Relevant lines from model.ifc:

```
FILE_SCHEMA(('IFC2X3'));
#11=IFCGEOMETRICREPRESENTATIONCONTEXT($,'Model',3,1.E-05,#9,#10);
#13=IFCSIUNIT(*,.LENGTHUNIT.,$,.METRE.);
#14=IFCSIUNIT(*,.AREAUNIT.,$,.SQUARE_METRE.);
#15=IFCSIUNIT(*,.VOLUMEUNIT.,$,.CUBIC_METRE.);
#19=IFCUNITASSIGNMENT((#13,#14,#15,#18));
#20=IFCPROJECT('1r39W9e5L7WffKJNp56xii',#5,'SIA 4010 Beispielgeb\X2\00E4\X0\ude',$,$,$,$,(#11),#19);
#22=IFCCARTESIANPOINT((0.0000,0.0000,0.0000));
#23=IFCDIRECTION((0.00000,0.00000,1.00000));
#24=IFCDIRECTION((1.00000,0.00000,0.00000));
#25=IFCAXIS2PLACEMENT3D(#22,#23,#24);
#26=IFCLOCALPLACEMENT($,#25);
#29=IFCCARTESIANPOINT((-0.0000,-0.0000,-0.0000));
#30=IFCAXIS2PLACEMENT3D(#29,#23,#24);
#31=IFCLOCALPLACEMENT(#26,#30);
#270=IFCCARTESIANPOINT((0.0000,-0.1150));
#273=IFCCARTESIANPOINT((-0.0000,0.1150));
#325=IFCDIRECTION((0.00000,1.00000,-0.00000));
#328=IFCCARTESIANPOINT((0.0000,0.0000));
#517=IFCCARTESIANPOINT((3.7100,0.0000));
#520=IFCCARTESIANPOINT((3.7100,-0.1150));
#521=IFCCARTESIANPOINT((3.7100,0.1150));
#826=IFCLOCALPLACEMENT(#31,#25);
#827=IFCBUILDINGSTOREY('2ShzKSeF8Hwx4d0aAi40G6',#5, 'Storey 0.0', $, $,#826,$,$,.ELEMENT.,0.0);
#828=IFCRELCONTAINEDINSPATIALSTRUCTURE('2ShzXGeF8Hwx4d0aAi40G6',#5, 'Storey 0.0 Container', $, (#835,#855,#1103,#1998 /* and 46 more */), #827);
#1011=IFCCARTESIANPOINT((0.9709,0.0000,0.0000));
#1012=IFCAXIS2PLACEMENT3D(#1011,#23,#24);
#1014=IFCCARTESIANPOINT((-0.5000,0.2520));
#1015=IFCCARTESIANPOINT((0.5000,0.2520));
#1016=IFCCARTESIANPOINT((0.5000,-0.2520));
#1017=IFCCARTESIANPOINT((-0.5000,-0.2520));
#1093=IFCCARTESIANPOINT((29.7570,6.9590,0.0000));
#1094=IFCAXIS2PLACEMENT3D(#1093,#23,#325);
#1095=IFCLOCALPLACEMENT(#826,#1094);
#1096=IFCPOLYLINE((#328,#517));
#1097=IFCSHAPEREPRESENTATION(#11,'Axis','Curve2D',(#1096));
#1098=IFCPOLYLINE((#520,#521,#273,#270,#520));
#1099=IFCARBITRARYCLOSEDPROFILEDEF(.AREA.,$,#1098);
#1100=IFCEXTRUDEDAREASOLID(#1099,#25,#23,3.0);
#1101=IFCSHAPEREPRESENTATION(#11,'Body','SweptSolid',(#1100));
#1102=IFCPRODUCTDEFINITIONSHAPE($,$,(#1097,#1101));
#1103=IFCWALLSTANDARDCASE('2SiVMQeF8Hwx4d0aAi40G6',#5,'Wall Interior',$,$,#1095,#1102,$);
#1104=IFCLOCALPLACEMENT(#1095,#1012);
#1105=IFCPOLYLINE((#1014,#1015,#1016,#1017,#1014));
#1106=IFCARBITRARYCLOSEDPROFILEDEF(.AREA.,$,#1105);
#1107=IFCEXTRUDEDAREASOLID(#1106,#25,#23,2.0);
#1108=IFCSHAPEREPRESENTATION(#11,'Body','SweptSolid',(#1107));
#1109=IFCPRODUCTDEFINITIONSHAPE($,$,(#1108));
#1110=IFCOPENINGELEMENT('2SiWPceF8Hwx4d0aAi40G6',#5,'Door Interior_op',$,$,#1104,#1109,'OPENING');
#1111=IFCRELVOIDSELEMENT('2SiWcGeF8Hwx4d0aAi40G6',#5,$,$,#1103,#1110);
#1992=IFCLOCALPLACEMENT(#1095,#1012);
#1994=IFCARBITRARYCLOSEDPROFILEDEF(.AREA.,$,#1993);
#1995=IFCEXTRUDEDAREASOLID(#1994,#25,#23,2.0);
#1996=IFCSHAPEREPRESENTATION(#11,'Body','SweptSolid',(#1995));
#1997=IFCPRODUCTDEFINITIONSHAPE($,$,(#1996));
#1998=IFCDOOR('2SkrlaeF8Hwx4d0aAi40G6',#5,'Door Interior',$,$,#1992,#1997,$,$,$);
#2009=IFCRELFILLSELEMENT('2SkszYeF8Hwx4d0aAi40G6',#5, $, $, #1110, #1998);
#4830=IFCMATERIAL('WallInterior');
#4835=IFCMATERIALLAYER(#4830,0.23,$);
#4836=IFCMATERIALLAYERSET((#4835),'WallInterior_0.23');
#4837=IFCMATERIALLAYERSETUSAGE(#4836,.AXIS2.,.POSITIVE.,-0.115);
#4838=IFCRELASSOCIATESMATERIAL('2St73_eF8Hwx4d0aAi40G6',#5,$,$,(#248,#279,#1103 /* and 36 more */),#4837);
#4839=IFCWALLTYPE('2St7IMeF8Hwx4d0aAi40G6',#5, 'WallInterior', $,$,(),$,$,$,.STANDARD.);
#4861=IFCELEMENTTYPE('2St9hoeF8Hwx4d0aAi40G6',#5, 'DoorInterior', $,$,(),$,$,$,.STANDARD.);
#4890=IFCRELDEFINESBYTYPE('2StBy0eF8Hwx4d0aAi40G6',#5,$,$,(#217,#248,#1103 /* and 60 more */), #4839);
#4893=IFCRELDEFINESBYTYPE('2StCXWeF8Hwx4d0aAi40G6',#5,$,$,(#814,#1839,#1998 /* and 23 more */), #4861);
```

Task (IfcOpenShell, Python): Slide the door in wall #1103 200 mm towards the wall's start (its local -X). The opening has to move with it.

```python
import ifcopenshell
import ifcopenshell.api.geometry
import ifcopenshell.util.placement
import ifcopenshell.util.unit

model = ifcopenshell.open("model.ifc")
unit_scale = ifcopenshell.util.unit.calculate_unit_scale(model)

door = model.by_guid("2SkrlaeF8Hwx4d0aAi40G6")
opening = door.FillsVoids[0].RelatingOpeningElement
wall = opening.VoidsElements[0].RelatingBuildingElement

wall_matrix = ifcopenshell.util.placement.get_local_placement(wall.ObjectPlacement)
shift = wall_matrix[:3, 0] * -0.2 / unit_scale
before = ifcopenshell.util.placement.get_local_placement(door.ObjectPlacement)[:3, 3].copy()

# The door is not placed relative to its opening, so move both.
for product in (opening, door):
    matrix = ifcopenshell.util.placement.get_local_placement(product.ObjectPlacement)
    matrix[:3, 3] += shift
    ifcopenshell.api.geometry.edit_object_placement(model, product=product, matrix=matrix, is_si=False)

after = ifcopenshell.util.placement.get_local_placement(door.ObjectPlacement)[:3, 3]
print("door moved by", (after - before).round(3) + 0.0)

model.write("model-out.ifc")
```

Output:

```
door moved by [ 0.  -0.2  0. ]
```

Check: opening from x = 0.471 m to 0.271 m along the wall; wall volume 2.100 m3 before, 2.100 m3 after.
